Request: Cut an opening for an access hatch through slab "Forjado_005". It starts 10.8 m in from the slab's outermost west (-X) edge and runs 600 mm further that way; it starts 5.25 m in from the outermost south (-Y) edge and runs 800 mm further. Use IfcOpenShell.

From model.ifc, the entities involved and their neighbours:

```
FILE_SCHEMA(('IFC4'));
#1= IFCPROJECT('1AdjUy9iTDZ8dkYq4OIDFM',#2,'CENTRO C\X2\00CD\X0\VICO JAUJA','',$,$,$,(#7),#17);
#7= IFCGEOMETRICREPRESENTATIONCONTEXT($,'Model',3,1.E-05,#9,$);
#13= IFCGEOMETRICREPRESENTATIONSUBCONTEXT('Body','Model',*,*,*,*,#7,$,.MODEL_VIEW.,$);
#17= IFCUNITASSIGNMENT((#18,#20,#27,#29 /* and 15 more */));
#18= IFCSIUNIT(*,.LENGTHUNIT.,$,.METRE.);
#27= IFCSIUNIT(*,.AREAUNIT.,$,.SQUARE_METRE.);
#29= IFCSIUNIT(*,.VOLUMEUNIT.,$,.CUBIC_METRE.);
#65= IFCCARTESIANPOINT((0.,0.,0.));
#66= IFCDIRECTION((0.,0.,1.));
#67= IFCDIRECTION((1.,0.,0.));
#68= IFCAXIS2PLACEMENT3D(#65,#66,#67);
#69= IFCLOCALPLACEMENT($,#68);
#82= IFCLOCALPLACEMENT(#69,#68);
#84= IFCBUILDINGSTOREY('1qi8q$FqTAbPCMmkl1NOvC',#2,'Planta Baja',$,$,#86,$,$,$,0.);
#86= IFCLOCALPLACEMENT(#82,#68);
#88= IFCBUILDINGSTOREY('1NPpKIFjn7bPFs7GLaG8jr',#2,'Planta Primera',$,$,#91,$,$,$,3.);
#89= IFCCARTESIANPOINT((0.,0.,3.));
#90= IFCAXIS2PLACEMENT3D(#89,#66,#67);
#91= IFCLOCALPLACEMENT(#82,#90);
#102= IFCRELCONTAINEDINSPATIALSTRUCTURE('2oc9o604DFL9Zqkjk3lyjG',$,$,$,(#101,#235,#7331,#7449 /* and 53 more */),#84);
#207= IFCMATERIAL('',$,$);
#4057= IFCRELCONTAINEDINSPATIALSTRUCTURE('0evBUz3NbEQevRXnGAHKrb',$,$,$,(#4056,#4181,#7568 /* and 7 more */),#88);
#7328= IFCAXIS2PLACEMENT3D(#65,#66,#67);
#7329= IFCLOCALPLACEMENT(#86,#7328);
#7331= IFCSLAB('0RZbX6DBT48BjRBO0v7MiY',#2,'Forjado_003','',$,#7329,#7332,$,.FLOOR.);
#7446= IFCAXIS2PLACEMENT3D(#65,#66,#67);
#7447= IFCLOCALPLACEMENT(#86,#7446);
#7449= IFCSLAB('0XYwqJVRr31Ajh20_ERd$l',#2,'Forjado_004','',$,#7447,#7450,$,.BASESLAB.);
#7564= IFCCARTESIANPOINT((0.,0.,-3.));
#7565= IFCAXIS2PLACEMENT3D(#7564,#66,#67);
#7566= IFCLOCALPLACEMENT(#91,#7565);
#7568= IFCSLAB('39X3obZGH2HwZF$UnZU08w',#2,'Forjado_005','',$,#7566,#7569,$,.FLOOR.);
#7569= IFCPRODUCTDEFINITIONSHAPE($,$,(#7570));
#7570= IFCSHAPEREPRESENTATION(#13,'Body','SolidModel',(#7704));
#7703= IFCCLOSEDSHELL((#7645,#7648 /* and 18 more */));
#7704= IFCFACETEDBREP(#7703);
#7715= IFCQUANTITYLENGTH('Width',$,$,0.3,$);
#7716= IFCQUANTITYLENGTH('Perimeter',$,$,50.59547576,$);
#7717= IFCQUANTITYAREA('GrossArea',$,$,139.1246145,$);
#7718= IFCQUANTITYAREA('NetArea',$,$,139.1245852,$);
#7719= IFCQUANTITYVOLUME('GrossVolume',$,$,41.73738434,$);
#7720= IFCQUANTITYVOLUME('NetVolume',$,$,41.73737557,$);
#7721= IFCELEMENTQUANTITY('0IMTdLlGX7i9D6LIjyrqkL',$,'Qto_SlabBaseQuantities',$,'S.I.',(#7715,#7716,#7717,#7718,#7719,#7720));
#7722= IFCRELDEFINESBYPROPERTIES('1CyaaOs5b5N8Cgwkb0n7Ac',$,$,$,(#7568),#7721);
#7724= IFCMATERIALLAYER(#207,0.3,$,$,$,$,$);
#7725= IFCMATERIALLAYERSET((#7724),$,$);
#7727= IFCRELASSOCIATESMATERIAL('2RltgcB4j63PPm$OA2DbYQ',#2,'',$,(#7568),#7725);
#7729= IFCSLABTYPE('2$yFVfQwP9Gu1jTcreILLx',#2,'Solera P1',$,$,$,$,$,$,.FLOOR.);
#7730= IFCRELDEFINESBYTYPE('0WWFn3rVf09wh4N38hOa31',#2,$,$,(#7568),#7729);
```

```python
import numpy as np
import ifcopenshell
import ifcopenshell.api.feature
import ifcopenshell.api.geometry
import ifcopenshell.api.pset
import ifcopenshell.api.root
import ifcopenshell.geom
import ifcopenshell.util.element
import ifcopenshell.util.placement
import ifcopenshell.util.representation
import ifcopenshell.util.shape
import ifcopenshell.util.unit

model = ifcopenshell.open("model.ifc")
unit_scale = ifcopenshell.util.unit.calculate_unit_scale(model)
area_scale = ifcopenshell.util.unit.calculate_unit_scale(model, "AREAUNIT")
volume_scale = ifcopenshell.util.unit.calculate_unit_scale(model, "VOLUMEUNIT")
settings = ifcopenshell.geom.settings()


def volume(element):
    """Net volume in cubic metres, openings subtracted."""
    shape = ifcopenshell.geom.create_shape(settings, element)
    return ifcopenshell.util.shape.get_volume(shape.geometry)


slab = model.by_guid("39X3obZGH2HwZF$UnZU08w")
before = volume(slab)

# Extent in the slab's own axes, in metres. The edges named are its -X and -Y sides.
slab_shape = ifcopenshell.geom.create_shape(settings, slab)
vertices = ifcopenshell.util.shape.get_vertices(slab_shape.geometry)
x_min, y_min, bottom = vertices.min(axis=0)
top = vertices[:, 2].max()

opening = ifcopenshell.api.root.create_entity(model, ifc_class="IfcOpeningElement", name="Access hatch opening", predefined_type="OPENING")
context = ifcopenshell.util.representation.get_context(model, "Model", "Body", "MODEL_VIEW")
width, depth = 0.6, 0.8
outline = [(0.0, 0.0), (width, 0.0), (width, depth), (0.0, depth), (0.0, 0.0)]
# Overshoot both faces by 50 mm so the cut is clean.
shape = ifcopenshell.api.geometry.add_slab_representation(
    model, context=context, depth=top - bottom + 0.1, polyline=outline
)
ifcopenshell.api.geometry.assign_representation(model, product=opening, representation=shape)

matrix = ifcopenshell.util.placement.get_local_placement(slab.ObjectPlacement)
matrix[:, 3] = matrix @ np.append(np.array([x_min + 10.8, y_min + 5.25, bottom - 0.05]) / unit_scale, 1.0)
ifcopenshell.api.geometry.edit_object_placement(model, product=opening, matrix=matrix, is_si=False)
ifcopenshell.api.feature.add_feature(model, feature=opening, element=slab)

after = volume(slab)

# Update the slab's stored quantities.
qto = model.by_id(ifcopenshell.util.element.get_pset(slab, "Qto_SlabBaseQuantities", should_inherit=False)["id"])
ifcopenshell.api.pset.edit_qto(model, qto=qto, properties={
    "NetArea": after / (top - bottom) / area_scale,
    "NetVolume": after / volume_scale,
})

print(f"slab volume {before:.3f} -> {after:.3f} m3")

model.write("model_updated.ifc")
```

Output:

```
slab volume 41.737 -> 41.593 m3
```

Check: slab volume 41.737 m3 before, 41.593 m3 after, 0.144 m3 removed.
